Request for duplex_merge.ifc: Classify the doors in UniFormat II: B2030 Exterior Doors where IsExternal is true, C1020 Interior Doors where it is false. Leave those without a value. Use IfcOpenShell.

First a look at what the model holds.

```python
import ifcopenshell
import ifcopenshell.util.element

model = ifcopenshell.open("duplex_merge.ifc")
print(model.schema)
print("classifications:", [c.Name for c in model.by_type("IfcClassification")])
values = [ifcopenshell.util.element.get_pset(e, "Pset_DoorCommon", "IsExternal") for e in model.by_type("IfcDoor")]
for value in (True, False, None):
    print("IsExternal", value, values.count(value))
```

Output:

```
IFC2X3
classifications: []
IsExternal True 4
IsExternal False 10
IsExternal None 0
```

```python
import ifcopenshell
import ifcopenshell.api.classification
import ifcopenshell.util.element

model = ifcopenshell.open("duplex_merge.ifc")

# IFC2X3 requires Source and Edition and has no link from the project to the system.
system = model.create_entity("IfcClassification", Source="ASTM", Edition="E1557", Name="UniFormat II")

doors = model.by_type("IfcDoor")
external = {e: ifcopenshell.util.element.get_pset(e, "Pset_DoorCommon", "IsExternal") for e in doors}
for flag, code, name in ((True, "B2030", "Exterior Doors"), (False, "C1020", "Interior Doors")):
    products = [e for e in doors if external[e] is flag]
    ifcopenshell.api.classification.add_reference(
        model, products=products, classification=system, identification=code, name=name
    )
    print(code, len(products))

model.write("duplex_merge-out.ifc")
```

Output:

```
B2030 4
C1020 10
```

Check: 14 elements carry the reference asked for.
